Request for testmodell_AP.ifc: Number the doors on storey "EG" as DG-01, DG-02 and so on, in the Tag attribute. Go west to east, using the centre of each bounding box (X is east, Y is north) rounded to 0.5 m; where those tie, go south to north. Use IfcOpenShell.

First a look at what the model holds.

```python
import ifcopenshell
import ifcopenshell.util.element
import ifcopenshell.util.placement

model = ifcopenshell.open("testmodell_AP.ifc")
print(model.schema)
storey = next(s for s in model.by_type("IfcBuildingStorey") if s.Name == "EG")
doors = [e for e in ifcopenshell.util.element.get_decomposition(storey) if e.is_a("IfcDoor")]
for e in sorted(doors, key=lambda e: e.id()):
    origin = ifcopenshell.util.placement.get_local_placement(e.ObjectPlacement)[:3, 3]
    print(e.id(), e.Tag, e.Name, origin.round(2) + 0.0, sep=" | ")
```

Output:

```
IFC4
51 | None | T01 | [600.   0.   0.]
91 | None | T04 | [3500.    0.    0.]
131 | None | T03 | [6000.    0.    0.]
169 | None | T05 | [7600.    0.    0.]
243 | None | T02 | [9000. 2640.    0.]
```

```python
import ifcopenshell
import ifcopenshell.geom
import ifcopenshell.util.element
import ifcopenshell.util.shape

model = ifcopenshell.open("testmodell_AP.ifc")
settings = ifcopenshell.geom.settings()
settings.set("use-world-coords", True)


def centre(element):
    shape = ifcopenshell.geom.create_shape(settings, element)
    return ifcopenshell.util.shape.get_bbox_centroid(shape.geometry)


storey = next(s for s in model.by_type("IfcBuildingStorey") if s.Name == "EG")
doors = [e for e in ifcopenshell.util.element.get_decomposition(storey) if e.is_a("IfcDoor")]

# Insertion points can sit at a corner or the storey origin, so sort by the geometry (in metres).
centres = {e: centre(e) for e in doors}
doors.sort(key=lambda e: (round(centres[e][0] / 0.5), centres[e][1]))

for i, e in enumerate(doors, start=1):
    number = f"DG-{i:02d}"
    e.Tag = number
    print(e.id(), number)

model.write("testmodell_AP_edited.ifc")
```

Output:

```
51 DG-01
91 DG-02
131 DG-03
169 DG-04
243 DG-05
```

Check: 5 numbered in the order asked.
